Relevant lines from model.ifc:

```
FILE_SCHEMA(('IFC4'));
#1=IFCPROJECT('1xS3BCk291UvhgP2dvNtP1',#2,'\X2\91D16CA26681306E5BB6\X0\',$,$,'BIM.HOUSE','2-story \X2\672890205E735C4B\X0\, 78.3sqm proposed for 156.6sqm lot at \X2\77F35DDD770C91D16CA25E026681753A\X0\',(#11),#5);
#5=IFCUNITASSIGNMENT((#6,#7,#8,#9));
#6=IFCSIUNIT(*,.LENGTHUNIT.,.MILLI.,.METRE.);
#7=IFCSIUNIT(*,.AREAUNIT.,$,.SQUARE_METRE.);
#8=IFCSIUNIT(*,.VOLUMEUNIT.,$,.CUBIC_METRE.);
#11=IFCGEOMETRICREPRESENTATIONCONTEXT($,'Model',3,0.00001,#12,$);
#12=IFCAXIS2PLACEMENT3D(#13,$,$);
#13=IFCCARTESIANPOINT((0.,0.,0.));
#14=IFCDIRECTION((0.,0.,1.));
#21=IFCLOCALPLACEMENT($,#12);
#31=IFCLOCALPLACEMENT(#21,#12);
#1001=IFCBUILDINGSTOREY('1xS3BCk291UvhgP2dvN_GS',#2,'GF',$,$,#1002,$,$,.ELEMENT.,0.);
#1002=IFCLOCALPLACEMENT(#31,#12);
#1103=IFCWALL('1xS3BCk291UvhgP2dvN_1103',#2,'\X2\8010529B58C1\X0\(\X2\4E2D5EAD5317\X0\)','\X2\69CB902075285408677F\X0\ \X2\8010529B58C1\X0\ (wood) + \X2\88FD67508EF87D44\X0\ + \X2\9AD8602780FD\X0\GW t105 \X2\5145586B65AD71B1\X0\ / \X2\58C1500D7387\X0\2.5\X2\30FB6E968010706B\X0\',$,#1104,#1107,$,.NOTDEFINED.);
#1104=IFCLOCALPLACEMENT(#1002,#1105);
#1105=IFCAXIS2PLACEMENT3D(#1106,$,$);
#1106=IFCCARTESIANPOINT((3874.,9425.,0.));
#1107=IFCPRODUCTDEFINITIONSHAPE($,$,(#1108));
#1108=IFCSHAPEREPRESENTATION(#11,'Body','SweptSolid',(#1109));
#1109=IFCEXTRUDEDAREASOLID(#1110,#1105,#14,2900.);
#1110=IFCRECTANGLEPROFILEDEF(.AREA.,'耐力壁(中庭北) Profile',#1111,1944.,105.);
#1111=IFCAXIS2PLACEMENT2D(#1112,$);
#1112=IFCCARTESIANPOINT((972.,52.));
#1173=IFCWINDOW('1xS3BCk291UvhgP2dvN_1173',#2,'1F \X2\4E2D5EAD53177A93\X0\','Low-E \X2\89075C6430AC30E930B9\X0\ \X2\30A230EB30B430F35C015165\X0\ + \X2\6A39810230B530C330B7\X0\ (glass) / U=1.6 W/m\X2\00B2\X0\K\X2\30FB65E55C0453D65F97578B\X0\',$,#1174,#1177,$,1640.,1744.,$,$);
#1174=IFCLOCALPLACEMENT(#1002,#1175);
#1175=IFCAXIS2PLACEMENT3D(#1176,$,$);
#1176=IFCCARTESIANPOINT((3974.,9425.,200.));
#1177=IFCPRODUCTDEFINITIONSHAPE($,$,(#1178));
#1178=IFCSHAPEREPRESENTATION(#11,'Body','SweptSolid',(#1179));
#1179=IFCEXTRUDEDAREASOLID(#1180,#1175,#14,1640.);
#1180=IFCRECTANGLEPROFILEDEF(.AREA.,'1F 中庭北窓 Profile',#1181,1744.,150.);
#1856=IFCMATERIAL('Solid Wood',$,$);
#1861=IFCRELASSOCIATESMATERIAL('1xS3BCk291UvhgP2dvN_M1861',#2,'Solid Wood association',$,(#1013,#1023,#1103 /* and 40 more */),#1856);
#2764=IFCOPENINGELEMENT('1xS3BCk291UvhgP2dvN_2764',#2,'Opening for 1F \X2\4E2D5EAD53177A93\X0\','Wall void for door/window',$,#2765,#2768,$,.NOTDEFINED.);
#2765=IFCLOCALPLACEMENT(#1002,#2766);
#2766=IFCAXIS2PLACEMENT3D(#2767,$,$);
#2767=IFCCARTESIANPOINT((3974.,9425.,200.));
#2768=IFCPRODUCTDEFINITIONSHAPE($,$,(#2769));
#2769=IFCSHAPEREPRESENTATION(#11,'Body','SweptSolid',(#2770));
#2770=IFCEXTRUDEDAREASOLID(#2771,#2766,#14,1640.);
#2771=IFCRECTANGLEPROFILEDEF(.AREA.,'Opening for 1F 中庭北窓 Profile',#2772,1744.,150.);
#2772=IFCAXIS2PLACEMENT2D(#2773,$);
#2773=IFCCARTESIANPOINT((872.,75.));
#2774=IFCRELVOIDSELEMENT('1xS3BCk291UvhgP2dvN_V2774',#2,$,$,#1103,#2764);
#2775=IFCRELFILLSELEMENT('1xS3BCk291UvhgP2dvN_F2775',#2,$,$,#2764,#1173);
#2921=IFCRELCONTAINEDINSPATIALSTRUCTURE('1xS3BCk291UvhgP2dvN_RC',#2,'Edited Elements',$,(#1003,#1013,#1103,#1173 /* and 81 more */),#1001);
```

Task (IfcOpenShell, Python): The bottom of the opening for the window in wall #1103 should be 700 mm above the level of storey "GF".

```python
import numpy as np
import ifcopenshell
import ifcopenshell.api.geometry
import ifcopenshell.geom
import ifcopenshell.util.element
import ifcopenshell.util.placement
import ifcopenshell.util.shape
import ifcopenshell.util.unit

model = ifcopenshell.open("model.ifc")
unit_scale = ifcopenshell.util.unit.calculate_unit_scale(model)

window = model.by_id(1173)
opening = window.FillsVoids[0].RelatingOpeningElement
storey = ifcopenshell.util.element.get_container(window, ifc_class="IfcBuildingStorey")
level = ifcopenshell.util.placement.get_local_placement(storey.ObjectPlacement)[2, 3]

# The opening's origin need not be at the sill, so measure its lowest point.
shape = ifcopenshell.geom.create_shape(ifcopenshell.geom.settings(), opening)
bottom = ifcopenshell.util.shape.get_shape_bottom_elevation(shape, shape.geometry) / unit_scale
dz = level + 700.0 - bottom

shift = np.array([0.0, 0.0, dz])
# The window is not placed relative to its opening, so move both.
for product in (opening, window):
    matrix = ifcopenshell.util.placement.get_local_placement(product.ObjectPlacement)
    matrix[:3, 3] += shift
    ifcopenshell.api.geometry.edit_object_placement(model, product=product, matrix=matrix, is_si=False)

print(f"moved by {dz * unit_scale:+.3f} m")

model.write("model_v2.ifc")
```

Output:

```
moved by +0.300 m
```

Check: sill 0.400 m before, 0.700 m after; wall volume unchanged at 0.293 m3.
